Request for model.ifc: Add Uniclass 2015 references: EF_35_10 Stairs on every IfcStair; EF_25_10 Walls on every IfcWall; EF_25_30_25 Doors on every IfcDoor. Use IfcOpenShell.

First a look at what the model holds.

```python
import ifcopenshell

model = ifcopenshell.open("model.ifc")
print(model.schema)
print("classifications:", [c.Name for c in model.by_type("IfcClassification")])
for ifc_class in ("IfcDoor", "IfcRoof", "IfcStair", "IfcWall", "IfcWindow"):
    print(ifc_class, len(model.by_type(ifc_class)))
```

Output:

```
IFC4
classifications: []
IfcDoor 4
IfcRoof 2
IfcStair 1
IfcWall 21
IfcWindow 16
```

```python
import ifcopenshell
import ifcopenshell.api.classification

model = ifcopenshell.open("model.ifc")

system = ifcopenshell.api.classification.add_classification(model, classification="Uniclass 2015")

codes = {
    "IfcStair": ("EF_35_10", "Stairs"),
    "IfcWall": ("EF_25_10", "Walls"),
    "IfcDoor": ("EF_25_30_25", "Doors"),
}
for ifc_class, (code, name) in codes.items():
    products = model.by_type(ifc_class)
    ifcopenshell.api.classification.add_reference(
        model, products=products, classification=system, identification=code, name=name
    )
    print(code, len(products))

model.write("model_updated.ifc")
```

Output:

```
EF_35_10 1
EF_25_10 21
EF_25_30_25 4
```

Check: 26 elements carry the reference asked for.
